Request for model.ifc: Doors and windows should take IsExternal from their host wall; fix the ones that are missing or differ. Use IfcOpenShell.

First a look at what the model holds.

```python
import ifcopenshell
import ifcopenshell.util.element

model = ifcopenshell.open("model.ifc")
print(model.schema)
seen = {}
for e in model.by_type("IfcDoor") + model.by_type("IfcWindow"):
    if not e.FillsVoids:
        continue
    host = e.FillsVoids[0].RelatingOpeningElement.VoidsElements[0].RelatingBuildingElement
    own = ifcopenshell.util.element.get_pset(e, f"Pset_{e.is_a()[3:].removesuffix('StandardCase')}Common", "IsExternal")
    wall = ifcopenshell.util.element.get_pset(host, "Pset_WallCommon", "IsExternal")
    seen[e.is_a(), own, wall] = seen.get((e.is_a(), own, wall), 0) + 1
for (cls, own, wall), count in sorted(seen.items(), key=str):
    print(count, cls, "IsExternal:", own, "| host wall:", wall)
```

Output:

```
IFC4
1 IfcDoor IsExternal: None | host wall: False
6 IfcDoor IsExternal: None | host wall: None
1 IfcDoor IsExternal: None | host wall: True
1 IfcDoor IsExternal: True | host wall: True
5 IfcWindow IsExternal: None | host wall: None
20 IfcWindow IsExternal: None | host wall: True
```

```python
import ifcopenshell
import ifcopenshell.api.pset
import ifcopenshell.util.element

model = ifcopenshell.open("model.ifc")

count = 0
for ifc_class, pset_name in (("IfcDoor", "Pset_DoorCommon"), ("IfcWindow", "Pset_WindowCommon")):
    for e in model.by_type(ifc_class):
        if not e.FillsVoids:
            continue
        host = e.FillsVoids[0].RelatingOpeningElement.VoidsElements[0].RelatingBuildingElement
        external = ifcopenshell.util.element.get_pset(host, "Pset_WallCommon", "IsExternal")
        if external is None or ifcopenshell.util.element.get_pset(e, pset_name, "IsExternal") == external:
            continue
        pset = ifcopenshell.api.pset.add_pset(model, product=e, name=pset_name)
        ifcopenshell.api.pset.edit_pset(model, pset=pset, properties={"IsExternal": external})
        count += 1

print(count, "updated")

model.write("model-out.ifc")
```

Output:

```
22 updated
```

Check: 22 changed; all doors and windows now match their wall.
